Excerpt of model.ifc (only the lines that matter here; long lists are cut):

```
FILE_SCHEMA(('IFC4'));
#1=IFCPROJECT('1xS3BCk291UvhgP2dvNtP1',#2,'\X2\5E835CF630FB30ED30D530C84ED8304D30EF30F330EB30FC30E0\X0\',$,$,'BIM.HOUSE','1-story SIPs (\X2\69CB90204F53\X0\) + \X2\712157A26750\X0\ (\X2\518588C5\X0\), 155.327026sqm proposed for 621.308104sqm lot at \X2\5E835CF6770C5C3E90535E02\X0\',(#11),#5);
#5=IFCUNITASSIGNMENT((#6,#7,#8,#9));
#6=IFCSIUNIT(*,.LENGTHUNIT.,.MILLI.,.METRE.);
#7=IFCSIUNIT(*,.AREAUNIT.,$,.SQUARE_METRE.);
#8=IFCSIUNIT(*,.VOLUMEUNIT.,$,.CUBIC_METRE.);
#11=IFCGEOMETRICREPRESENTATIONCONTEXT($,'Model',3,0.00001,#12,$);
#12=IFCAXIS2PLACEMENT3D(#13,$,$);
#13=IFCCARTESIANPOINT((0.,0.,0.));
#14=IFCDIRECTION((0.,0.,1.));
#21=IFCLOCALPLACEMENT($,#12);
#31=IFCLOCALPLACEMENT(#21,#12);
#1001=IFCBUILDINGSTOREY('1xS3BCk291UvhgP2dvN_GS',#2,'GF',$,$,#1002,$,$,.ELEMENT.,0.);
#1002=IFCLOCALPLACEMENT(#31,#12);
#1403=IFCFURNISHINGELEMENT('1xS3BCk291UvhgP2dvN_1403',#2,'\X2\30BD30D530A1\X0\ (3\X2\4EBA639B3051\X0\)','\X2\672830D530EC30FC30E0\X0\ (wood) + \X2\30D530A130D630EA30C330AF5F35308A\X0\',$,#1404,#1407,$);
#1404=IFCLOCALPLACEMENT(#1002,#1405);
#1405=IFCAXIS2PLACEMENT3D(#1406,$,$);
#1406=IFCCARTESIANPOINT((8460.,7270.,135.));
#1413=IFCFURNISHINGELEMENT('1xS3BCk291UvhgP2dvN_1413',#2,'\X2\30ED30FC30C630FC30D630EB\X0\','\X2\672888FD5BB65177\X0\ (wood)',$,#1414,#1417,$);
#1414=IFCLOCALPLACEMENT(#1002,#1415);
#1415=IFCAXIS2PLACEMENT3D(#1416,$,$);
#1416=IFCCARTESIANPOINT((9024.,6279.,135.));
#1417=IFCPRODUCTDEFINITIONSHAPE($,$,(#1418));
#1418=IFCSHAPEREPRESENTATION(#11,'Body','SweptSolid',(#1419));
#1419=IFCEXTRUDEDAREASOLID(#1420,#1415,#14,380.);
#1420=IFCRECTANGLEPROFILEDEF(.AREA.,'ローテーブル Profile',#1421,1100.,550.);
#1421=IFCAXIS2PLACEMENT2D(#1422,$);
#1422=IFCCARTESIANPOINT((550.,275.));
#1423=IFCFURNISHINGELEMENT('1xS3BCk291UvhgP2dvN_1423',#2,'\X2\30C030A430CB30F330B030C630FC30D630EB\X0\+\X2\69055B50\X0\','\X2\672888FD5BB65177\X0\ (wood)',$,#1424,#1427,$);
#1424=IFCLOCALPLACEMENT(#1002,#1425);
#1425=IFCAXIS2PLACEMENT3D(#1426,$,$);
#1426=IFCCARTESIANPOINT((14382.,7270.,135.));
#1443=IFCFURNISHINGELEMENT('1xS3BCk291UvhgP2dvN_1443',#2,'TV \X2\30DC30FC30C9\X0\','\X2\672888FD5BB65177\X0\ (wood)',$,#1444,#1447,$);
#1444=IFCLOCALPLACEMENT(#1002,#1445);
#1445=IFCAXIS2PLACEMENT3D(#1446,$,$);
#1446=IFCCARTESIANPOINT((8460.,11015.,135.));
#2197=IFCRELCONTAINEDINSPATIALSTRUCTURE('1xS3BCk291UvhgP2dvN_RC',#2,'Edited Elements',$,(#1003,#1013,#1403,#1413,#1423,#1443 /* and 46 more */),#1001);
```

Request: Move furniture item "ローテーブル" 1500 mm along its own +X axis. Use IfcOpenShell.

```python
import ifcopenshell
import ifcopenshell.api.geometry
import ifcopenshell.util.placement
import ifcopenshell.util.unit

model = ifcopenshell.open("model.ifc")
unit_scale = ifcopenshell.util.unit.calculate_unit_scale(model)

item = model.by_guid("1xS3BCk291UvhgP2dvN_1413")
matrix = ifcopenshell.util.placement.get_local_placement(item.ObjectPlacement)
matrix[:3, 3] += matrix[:3, 0] * 1.5 / unit_scale
ifcopenshell.api.geometry.edit_object_placement(model, product=item, matrix=matrix, is_si=False)

print(ifcopenshell.util.placement.get_local_placement(item.ObjectPlacement).round(3) + 0.0)

model.write("model_updated.ifc")
```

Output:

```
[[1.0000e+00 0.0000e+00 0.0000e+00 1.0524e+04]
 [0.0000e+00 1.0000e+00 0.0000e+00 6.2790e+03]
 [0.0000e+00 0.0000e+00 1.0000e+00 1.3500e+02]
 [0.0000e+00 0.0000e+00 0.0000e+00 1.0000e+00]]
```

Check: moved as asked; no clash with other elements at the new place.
